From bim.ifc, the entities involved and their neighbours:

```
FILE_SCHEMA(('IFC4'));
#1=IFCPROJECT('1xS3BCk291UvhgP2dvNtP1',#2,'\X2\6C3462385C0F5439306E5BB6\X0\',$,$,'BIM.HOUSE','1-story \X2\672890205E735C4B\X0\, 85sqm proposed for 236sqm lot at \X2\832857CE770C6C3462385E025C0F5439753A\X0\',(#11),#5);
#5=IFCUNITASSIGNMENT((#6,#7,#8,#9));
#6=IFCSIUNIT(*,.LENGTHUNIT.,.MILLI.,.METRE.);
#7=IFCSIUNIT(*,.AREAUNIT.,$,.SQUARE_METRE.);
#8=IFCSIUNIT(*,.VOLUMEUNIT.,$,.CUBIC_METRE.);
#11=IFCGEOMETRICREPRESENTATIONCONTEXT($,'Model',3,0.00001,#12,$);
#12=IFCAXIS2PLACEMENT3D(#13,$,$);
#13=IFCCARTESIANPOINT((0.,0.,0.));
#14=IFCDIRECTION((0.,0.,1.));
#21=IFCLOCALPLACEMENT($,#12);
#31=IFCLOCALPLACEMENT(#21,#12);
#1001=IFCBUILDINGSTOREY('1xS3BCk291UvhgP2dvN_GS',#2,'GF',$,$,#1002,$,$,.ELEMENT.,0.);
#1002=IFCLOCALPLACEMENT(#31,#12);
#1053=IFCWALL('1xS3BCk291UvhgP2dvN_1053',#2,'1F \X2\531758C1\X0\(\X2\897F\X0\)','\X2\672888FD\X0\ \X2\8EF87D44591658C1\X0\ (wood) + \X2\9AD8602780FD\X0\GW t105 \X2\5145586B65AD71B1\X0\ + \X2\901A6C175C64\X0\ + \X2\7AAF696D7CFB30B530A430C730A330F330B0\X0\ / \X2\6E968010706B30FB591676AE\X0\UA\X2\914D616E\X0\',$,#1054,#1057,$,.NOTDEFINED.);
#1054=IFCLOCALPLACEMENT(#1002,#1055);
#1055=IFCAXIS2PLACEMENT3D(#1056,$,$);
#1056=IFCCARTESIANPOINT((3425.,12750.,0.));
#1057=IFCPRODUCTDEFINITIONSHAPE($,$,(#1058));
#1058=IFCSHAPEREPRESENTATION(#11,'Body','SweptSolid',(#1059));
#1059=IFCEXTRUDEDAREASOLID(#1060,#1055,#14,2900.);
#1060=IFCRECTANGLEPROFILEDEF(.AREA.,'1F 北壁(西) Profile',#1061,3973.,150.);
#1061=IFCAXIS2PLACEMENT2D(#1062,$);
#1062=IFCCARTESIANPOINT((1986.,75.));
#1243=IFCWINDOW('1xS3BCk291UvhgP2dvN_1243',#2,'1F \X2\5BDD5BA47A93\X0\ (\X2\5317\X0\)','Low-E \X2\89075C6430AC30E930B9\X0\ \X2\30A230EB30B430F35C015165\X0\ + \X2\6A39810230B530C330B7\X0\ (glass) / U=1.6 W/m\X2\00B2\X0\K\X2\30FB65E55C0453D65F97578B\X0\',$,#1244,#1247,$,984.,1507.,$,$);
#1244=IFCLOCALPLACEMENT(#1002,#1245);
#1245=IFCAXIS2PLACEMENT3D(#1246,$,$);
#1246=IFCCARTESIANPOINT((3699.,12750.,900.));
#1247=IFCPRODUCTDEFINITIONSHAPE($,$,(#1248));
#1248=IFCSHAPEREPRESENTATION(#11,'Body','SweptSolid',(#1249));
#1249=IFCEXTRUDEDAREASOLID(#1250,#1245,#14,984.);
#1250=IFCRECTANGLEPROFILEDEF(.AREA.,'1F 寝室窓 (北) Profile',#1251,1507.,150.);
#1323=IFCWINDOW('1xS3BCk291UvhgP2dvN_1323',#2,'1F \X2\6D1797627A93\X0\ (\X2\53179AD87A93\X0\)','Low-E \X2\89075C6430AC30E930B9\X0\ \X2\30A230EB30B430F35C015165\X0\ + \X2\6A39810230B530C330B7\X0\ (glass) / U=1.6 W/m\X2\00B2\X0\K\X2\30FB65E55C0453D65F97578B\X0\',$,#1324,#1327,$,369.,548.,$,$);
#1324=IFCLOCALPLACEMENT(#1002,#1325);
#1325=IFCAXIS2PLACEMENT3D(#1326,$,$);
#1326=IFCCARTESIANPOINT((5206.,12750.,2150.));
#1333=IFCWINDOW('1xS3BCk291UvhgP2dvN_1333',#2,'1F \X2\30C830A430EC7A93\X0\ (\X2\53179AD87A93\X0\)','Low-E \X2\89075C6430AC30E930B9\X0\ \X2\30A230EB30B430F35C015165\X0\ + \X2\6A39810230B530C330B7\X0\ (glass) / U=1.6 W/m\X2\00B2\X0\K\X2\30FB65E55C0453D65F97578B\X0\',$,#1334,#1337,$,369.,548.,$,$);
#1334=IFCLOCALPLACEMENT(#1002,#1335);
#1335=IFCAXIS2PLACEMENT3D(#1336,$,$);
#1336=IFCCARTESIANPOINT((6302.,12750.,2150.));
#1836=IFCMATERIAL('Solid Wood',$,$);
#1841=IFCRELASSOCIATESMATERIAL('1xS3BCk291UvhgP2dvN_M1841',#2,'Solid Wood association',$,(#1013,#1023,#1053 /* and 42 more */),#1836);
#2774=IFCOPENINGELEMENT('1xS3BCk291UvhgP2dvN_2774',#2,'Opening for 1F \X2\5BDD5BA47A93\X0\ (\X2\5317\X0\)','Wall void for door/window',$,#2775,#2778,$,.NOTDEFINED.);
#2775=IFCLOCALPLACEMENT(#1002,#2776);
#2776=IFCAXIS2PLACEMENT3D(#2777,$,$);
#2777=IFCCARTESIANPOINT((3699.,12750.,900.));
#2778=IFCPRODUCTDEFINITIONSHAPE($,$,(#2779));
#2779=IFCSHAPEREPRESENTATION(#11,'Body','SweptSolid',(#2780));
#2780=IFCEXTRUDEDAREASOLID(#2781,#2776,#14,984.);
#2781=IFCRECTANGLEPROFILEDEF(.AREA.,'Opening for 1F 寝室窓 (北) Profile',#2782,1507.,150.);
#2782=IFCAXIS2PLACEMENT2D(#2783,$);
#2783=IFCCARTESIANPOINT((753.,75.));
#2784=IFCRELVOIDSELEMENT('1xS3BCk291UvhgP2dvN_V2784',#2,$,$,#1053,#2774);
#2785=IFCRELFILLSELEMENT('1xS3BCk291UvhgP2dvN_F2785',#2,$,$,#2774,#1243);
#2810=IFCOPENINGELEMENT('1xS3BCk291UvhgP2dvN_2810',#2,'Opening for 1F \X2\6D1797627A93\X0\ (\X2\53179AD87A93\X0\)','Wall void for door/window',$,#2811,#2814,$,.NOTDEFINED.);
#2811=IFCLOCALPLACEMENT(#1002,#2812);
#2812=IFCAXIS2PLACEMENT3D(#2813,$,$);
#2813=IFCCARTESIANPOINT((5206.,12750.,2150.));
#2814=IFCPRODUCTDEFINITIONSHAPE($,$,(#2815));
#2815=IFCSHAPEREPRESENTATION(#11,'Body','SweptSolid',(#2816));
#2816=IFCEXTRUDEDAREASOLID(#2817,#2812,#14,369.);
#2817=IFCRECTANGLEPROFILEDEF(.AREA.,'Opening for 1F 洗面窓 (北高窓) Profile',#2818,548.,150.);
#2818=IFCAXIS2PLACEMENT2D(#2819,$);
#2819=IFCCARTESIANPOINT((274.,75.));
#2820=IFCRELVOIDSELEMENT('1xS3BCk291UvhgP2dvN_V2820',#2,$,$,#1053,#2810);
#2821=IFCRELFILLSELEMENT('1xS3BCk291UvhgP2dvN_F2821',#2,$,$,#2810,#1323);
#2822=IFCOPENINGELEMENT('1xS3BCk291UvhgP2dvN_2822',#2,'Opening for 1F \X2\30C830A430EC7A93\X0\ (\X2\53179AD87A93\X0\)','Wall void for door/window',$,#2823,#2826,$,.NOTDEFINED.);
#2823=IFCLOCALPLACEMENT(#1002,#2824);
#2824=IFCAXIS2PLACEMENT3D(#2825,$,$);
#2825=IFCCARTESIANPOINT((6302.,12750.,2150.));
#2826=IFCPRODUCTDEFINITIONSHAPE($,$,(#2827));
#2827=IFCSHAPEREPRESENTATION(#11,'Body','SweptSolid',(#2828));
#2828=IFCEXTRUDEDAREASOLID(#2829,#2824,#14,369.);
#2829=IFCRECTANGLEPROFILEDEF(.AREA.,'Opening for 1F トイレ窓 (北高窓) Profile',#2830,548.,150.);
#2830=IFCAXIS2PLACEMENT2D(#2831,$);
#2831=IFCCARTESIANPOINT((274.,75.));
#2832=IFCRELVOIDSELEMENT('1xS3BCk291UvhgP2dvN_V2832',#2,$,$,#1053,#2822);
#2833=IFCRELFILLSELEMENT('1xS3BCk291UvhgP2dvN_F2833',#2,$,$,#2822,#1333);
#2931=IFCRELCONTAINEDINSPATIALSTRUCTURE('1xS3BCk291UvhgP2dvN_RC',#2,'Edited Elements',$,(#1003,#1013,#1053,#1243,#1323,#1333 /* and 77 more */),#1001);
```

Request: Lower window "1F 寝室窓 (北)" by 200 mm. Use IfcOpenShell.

```python
import numpy as np
import ifcopenshell
import ifcopenshell.api.geometry
import ifcopenshell.util.placement
import ifcopenshell.util.unit

model = ifcopenshell.open("bim.ifc")
unit_scale = ifcopenshell.util.unit.calculate_unit_scale(model)

window = model.by_id(1243)
opening = window.FillsVoids[0].RelatingOpeningElement
dz = -200.0

shift = np.array([0.0, 0.0, dz])
# The window is not placed relative to its opening, so move both.
for product in (opening, window):
    matrix = ifcopenshell.util.placement.get_local_placement(product.ObjectPlacement)
    matrix[:3, 3] += shift
    ifcopenshell.api.geometry.edit_object_placement(model, product=product, matrix=matrix, is_si=False)

print(f"moved by {dz * unit_scale:+.3f} m")

model.write("bim_rev.ifc")
```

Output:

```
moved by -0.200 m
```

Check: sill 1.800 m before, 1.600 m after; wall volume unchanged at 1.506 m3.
